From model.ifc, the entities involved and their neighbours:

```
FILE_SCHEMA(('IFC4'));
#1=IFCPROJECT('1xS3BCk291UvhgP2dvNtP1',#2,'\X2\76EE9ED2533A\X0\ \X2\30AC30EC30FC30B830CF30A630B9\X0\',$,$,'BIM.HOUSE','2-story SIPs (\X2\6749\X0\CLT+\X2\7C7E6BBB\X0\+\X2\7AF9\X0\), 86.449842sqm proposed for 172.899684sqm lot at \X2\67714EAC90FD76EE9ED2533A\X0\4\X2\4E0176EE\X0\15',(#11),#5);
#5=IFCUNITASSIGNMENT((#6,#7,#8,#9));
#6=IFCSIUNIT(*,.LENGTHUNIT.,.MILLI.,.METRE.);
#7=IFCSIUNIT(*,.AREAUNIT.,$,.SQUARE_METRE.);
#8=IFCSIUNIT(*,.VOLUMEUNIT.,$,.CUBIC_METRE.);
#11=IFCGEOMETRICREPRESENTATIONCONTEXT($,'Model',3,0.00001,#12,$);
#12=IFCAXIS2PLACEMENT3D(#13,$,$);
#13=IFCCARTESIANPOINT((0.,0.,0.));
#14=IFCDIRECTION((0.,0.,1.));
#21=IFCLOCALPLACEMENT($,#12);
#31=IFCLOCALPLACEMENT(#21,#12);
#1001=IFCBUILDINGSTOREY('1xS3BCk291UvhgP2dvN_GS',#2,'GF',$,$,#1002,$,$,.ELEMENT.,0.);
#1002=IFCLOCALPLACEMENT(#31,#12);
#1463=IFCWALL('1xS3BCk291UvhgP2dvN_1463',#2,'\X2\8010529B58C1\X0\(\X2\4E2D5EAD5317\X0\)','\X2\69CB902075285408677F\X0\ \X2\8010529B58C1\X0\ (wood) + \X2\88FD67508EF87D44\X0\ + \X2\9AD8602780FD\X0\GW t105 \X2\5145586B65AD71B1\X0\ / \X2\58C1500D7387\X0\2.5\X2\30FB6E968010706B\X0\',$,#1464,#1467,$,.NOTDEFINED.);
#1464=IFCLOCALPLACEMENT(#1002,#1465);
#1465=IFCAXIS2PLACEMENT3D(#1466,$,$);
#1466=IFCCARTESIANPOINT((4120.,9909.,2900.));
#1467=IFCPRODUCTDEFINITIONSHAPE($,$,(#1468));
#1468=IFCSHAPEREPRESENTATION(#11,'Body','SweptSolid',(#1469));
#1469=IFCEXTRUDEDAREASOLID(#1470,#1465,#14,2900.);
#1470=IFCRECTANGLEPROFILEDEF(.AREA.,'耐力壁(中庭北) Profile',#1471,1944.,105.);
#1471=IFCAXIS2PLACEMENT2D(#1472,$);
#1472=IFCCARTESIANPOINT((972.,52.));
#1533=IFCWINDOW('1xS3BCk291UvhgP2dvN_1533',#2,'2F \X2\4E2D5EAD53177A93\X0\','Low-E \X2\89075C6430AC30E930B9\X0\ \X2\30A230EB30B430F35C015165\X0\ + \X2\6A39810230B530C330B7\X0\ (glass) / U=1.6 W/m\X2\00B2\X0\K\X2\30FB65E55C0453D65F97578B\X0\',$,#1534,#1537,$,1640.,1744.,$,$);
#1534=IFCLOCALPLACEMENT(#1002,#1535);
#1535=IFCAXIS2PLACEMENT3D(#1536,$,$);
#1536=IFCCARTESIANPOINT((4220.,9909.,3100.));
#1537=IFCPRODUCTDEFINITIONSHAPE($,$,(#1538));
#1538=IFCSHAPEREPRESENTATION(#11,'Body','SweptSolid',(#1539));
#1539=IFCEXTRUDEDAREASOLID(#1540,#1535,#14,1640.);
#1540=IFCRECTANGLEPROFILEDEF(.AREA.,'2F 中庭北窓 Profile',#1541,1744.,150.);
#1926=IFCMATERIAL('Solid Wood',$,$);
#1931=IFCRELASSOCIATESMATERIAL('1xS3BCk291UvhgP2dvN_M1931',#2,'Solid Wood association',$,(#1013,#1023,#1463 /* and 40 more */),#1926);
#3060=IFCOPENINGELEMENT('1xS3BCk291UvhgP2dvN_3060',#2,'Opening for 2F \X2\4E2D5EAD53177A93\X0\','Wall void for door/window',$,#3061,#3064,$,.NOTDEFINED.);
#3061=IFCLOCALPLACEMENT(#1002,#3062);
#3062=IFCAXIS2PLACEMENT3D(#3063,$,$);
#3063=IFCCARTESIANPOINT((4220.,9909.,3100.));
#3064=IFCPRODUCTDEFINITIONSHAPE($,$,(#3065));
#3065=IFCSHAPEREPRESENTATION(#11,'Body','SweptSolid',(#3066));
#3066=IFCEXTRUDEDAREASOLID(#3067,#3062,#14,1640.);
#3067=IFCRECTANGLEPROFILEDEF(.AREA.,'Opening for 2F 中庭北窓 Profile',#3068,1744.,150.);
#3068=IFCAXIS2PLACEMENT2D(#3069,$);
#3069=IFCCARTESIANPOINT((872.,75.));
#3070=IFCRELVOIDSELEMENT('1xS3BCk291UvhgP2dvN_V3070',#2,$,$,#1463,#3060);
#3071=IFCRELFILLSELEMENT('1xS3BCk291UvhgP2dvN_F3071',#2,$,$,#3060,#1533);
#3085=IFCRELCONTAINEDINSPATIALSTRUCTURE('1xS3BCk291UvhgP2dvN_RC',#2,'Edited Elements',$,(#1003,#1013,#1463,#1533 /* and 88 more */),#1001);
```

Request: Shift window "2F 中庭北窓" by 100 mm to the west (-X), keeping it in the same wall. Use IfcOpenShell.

```python
import ifcopenshell
import ifcopenshell.api.geometry
import ifcopenshell.util.placement
import ifcopenshell.util.unit

model = ifcopenshell.open("model.ifc")
unit_scale = ifcopenshell.util.unit.calculate_unit_scale(model)

window = model.by_id(1533)
opening = window.FillsVoids[0].RelatingOpeningElement
wall = opening.VoidsElements[0].RelatingBuildingElement

wall_matrix = ifcopenshell.util.placement.get_local_placement(wall.ObjectPlacement)
shift = wall_matrix[:3, 0] * -0.1 / unit_scale
before = ifcopenshell.util.placement.get_local_placement(window.ObjectPlacement)[:3, 3].copy()

# The window is not placed relative to its opening, so move both.
for product in (opening, window):
    matrix = ifcopenshell.util.placement.get_local_placement(product.ObjectPlacement)
    matrix[:3, 3] += shift
    ifcopenshell.api.geometry.edit_object_placement(model, product=product, matrix=matrix, is_si=False)

after = ifcopenshell.util.placement.get_local_placement(window.ObjectPlacement)[:3, 3]
print("window moved by", (after - before).round(3) + 0.0)

model.write("model_edited.ifc")
```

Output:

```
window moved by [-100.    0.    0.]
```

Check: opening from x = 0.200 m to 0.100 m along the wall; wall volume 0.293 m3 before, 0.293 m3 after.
